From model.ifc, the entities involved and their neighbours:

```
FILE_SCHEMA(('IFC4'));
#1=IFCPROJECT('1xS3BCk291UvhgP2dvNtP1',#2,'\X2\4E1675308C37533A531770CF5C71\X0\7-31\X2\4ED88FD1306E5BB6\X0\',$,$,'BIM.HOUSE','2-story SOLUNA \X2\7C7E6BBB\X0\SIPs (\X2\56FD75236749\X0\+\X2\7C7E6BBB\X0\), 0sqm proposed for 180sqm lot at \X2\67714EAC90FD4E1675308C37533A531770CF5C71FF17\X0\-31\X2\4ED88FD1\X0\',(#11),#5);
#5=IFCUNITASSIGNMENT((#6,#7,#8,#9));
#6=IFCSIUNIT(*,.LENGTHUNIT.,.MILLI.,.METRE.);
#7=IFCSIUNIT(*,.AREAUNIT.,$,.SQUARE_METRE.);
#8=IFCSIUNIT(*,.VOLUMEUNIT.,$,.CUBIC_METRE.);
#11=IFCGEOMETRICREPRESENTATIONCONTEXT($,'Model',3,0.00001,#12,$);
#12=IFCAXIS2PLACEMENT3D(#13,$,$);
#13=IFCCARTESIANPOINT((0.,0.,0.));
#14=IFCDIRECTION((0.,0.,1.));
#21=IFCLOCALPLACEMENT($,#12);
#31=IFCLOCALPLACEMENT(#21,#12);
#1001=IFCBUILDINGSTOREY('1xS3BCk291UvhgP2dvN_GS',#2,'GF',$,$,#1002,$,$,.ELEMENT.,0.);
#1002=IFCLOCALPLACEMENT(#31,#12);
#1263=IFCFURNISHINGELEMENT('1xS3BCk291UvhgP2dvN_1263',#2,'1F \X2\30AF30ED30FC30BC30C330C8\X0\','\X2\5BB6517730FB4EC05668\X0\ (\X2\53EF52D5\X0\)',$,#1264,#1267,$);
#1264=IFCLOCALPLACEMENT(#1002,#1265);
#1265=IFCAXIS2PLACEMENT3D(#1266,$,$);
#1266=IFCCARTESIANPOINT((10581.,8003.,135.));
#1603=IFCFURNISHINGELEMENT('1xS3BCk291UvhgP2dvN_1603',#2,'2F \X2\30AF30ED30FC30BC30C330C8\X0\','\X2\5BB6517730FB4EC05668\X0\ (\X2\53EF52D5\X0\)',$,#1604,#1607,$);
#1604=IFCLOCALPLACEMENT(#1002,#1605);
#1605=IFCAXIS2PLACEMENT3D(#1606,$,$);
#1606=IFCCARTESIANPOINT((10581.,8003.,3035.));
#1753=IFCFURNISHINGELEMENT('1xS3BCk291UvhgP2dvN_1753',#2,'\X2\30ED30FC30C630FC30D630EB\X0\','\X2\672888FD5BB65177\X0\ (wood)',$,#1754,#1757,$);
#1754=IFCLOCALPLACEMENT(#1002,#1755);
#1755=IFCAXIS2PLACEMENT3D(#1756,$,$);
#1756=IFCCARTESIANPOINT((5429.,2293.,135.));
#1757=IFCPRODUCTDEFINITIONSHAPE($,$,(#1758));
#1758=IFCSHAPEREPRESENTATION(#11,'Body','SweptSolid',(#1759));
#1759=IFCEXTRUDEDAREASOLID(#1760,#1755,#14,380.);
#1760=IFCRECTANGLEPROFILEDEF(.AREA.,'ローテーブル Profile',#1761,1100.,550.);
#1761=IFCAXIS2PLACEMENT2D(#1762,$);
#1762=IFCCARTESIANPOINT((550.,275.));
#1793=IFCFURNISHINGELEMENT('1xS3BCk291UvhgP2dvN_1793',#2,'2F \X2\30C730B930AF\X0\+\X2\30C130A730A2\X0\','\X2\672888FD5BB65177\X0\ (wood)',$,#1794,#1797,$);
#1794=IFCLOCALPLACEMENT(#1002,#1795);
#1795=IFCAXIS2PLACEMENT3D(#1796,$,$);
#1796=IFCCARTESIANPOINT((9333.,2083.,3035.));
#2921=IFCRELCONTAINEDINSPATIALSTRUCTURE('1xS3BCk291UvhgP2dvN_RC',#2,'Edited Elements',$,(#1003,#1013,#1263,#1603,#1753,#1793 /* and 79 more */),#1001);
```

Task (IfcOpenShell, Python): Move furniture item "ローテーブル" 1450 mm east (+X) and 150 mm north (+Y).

```python
import ifcopenshell
import ifcopenshell.api.geometry
import ifcopenshell.util.placement

model = ifcopenshell.open("model.ifc")

item = model.by_id(1753)
matrix = ifcopenshell.util.placement.get_local_placement(item.ObjectPlacement)
matrix[0, 3] += 1450.0
matrix[1, 3] += 150.0
ifcopenshell.api.geometry.edit_object_placement(model, product=item, matrix=matrix, is_si=False)

print(ifcopenshell.util.placement.get_local_placement(item.ObjectPlacement).round(3) + 0.0)

model.write("model-out.ifc")
```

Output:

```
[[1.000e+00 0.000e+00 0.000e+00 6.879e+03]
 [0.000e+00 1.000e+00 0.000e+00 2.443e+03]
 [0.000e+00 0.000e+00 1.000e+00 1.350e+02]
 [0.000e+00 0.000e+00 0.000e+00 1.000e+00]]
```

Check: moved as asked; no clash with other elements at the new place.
